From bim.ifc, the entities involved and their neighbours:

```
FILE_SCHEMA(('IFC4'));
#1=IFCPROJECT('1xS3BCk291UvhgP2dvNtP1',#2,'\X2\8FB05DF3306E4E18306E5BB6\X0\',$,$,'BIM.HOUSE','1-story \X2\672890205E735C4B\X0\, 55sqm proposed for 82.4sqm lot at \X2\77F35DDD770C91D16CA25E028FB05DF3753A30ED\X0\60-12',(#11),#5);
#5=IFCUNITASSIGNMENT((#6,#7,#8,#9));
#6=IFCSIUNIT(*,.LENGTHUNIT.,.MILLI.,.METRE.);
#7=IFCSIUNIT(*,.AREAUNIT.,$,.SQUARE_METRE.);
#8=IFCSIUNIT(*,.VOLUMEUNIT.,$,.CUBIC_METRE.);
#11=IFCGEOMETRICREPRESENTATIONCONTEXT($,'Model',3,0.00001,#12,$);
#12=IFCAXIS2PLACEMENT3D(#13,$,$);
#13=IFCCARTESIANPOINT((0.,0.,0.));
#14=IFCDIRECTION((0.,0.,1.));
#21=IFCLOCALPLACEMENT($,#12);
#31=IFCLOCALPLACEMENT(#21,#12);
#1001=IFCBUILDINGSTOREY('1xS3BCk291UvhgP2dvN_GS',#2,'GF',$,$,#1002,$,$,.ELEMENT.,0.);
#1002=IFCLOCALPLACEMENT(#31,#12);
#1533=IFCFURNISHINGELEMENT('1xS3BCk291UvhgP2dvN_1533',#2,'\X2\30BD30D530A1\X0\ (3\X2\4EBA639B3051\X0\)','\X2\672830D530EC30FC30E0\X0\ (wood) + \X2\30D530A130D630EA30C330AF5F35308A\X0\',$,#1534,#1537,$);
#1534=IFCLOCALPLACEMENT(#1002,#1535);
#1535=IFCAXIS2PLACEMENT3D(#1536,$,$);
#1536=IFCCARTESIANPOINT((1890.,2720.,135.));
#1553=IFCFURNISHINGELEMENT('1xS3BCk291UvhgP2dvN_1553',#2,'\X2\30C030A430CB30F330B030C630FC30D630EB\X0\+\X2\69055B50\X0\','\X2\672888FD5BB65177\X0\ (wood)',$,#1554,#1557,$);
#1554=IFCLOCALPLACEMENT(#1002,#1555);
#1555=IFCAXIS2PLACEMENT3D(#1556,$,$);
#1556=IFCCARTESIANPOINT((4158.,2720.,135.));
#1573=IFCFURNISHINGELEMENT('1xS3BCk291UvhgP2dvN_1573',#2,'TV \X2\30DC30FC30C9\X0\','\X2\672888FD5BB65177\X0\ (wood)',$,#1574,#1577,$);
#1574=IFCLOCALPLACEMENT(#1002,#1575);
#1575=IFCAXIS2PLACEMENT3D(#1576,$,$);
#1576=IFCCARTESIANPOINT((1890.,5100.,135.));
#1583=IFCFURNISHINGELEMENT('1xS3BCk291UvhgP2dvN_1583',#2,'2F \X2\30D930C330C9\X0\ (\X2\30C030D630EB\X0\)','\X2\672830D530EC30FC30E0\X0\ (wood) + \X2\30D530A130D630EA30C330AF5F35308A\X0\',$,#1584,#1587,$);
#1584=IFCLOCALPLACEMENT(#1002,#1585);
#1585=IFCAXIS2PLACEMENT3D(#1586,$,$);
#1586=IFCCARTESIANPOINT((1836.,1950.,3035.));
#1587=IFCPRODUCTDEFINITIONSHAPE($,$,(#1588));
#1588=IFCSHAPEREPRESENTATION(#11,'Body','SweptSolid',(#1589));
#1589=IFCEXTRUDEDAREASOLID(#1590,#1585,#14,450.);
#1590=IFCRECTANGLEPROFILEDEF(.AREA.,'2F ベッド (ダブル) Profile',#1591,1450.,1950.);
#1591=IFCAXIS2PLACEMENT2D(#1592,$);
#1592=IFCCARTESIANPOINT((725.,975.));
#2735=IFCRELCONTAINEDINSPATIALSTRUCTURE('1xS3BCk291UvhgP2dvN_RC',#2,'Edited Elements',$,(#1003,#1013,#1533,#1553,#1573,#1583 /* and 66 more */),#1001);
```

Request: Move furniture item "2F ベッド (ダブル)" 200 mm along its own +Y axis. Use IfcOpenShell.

```python
import ifcopenshell
import ifcopenshell.api.geometry
import ifcopenshell.util.placement
import ifcopenshell.util.unit

model = ifcopenshell.open("bim.ifc")
unit_scale = ifcopenshell.util.unit.calculate_unit_scale(model)

item = model.by_guid("1xS3BCk291UvhgP2dvN_1583")
matrix = ifcopenshell.util.placement.get_local_placement(item.ObjectPlacement)
matrix[:3, 3] += matrix[:3, 1] * 0.2 / unit_scale
ifcopenshell.api.geometry.edit_object_placement(model, product=item, matrix=matrix, is_si=False)

print(ifcopenshell.util.placement.get_local_placement(item.ObjectPlacement).round(3) + 0.0)

model.write("bim-out.ifc")
```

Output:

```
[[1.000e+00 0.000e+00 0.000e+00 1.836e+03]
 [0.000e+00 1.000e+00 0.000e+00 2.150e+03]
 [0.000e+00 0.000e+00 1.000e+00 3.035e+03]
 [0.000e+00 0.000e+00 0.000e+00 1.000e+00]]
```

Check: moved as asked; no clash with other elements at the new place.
